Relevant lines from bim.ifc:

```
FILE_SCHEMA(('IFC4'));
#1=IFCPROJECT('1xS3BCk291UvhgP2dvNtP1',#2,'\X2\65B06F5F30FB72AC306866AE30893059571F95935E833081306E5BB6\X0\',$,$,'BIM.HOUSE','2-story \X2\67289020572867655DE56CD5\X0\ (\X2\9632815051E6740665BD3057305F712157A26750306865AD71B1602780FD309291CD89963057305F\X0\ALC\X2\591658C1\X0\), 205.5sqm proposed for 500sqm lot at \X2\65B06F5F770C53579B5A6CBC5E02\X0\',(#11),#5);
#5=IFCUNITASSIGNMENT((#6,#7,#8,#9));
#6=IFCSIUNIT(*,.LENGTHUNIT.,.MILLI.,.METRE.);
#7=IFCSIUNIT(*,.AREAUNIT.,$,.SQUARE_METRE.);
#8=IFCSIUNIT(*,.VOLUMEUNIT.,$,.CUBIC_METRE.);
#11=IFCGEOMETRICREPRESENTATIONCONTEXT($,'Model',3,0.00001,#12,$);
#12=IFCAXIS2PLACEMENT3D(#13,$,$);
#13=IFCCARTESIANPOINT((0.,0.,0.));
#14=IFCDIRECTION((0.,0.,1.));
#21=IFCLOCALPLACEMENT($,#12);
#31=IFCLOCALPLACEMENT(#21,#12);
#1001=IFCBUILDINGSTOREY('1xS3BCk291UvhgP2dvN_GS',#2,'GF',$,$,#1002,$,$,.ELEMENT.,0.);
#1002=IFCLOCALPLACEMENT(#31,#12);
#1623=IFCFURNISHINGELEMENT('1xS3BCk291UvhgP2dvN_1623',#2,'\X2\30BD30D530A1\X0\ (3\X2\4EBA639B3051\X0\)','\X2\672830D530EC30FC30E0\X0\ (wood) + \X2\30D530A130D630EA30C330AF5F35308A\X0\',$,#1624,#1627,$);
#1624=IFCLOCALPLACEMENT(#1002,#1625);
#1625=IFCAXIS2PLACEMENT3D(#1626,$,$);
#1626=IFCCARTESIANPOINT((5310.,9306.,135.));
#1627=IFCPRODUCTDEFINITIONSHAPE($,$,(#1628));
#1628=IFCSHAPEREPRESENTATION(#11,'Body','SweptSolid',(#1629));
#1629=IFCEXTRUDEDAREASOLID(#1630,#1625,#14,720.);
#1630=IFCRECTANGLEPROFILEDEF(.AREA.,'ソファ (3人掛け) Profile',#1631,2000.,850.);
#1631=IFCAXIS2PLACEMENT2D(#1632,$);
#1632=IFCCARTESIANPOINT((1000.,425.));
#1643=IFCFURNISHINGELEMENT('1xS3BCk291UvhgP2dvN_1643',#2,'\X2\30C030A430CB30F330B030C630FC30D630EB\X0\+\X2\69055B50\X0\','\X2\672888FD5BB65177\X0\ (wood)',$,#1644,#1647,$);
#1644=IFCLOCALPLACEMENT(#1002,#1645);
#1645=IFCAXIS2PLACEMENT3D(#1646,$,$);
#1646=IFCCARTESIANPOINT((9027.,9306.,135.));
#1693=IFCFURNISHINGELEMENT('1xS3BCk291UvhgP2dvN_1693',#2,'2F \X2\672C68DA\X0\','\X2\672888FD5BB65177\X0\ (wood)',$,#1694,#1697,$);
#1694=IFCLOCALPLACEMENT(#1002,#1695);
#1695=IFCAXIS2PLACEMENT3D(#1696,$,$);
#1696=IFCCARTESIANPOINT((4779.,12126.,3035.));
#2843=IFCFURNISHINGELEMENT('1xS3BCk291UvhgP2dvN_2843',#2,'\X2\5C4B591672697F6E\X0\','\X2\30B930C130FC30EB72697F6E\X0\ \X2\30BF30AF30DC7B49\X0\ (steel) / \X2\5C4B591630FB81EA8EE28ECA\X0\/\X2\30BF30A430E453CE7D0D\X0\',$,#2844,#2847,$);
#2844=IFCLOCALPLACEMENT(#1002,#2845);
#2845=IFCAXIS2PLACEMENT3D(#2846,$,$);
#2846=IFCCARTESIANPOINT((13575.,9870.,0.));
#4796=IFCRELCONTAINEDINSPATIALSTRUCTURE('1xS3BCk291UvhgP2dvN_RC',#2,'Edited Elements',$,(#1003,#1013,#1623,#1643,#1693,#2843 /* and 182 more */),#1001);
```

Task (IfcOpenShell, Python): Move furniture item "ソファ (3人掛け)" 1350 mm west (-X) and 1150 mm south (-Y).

```python
import ifcopenshell
import ifcopenshell.api.geometry
import ifcopenshell.util.placement

model = ifcopenshell.open("bim.ifc")

item = model.by_guid("1xS3BCk291UvhgP2dvN_1623")
matrix = ifcopenshell.util.placement.get_local_placement(item.ObjectPlacement)
matrix[0, 3] -= 1350.0
matrix[1, 3] -= 1150.0
ifcopenshell.api.geometry.edit_object_placement(model, product=item, matrix=matrix, is_si=False)

print(ifcopenshell.util.placement.get_local_placement(item.ObjectPlacement).round(3) + 0.0)

model.write("bim_updated.ifc")
```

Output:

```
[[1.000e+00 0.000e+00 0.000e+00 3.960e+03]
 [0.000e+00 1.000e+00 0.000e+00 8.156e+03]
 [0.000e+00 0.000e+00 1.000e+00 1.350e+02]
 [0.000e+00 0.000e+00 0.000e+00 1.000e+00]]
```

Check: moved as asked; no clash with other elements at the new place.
